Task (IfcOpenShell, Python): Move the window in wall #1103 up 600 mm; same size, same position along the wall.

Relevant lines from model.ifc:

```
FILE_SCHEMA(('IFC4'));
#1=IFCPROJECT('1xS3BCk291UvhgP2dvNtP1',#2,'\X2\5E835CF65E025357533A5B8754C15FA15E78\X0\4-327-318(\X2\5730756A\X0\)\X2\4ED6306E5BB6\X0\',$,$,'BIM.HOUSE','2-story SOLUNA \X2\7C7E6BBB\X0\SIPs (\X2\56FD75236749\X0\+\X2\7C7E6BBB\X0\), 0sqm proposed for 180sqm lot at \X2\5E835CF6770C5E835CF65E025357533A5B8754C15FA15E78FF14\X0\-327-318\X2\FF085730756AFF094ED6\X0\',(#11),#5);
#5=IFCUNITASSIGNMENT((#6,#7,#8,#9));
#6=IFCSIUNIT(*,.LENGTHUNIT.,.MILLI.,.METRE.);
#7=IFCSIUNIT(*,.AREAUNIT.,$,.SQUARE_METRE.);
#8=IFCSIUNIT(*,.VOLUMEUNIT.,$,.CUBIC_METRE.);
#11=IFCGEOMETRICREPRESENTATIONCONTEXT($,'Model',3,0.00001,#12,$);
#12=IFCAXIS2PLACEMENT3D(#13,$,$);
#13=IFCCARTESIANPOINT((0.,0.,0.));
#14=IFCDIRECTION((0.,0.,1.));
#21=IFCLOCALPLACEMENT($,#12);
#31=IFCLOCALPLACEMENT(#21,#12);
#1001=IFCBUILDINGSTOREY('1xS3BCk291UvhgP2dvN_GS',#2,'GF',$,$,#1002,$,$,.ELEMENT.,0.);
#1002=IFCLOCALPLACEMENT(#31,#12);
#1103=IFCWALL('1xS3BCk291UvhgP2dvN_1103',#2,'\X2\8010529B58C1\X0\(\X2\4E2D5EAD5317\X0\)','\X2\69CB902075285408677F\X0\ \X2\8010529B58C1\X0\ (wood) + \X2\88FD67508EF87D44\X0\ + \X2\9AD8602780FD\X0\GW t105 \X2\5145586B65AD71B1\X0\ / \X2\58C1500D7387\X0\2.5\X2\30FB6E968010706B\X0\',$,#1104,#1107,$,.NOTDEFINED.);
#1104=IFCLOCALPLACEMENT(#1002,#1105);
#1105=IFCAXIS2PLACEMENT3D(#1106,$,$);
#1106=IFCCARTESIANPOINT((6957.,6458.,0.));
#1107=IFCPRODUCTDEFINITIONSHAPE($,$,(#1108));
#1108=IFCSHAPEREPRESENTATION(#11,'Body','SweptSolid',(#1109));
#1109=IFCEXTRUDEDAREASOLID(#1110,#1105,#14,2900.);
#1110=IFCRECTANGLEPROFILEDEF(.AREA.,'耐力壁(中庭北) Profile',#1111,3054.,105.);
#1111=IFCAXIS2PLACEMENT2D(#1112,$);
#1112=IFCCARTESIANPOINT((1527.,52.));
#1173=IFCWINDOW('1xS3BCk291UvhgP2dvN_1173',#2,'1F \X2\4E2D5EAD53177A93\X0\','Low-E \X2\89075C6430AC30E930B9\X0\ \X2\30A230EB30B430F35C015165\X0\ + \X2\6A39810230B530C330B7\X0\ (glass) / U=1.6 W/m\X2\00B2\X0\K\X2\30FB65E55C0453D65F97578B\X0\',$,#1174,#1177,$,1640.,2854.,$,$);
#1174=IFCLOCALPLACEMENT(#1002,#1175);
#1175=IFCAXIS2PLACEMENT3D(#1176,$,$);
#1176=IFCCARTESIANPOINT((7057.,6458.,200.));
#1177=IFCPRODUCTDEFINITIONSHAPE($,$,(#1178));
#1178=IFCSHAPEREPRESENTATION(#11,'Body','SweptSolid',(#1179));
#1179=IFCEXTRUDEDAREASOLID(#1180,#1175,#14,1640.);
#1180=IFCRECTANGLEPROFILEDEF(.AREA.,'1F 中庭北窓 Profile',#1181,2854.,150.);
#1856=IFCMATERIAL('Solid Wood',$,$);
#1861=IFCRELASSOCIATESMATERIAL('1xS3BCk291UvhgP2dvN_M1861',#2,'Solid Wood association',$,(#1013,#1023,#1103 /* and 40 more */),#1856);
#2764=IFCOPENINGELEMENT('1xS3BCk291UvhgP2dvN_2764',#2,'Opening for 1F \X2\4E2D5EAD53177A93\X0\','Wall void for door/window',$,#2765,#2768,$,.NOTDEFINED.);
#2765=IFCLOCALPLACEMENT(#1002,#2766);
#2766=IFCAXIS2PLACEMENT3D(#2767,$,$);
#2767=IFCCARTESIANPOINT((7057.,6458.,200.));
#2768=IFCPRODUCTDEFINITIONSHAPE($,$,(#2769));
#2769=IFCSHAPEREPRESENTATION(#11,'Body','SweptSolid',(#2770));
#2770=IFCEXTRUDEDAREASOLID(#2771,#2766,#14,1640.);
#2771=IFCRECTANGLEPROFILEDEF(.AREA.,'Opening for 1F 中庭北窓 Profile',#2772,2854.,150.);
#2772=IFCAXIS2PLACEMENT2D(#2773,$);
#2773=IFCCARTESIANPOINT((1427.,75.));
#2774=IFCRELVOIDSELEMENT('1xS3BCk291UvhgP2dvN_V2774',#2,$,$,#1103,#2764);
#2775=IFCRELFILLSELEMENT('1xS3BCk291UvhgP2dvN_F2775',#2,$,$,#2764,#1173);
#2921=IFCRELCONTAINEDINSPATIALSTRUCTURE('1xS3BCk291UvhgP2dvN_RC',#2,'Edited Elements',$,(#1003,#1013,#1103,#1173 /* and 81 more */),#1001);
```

```python
import numpy as np
import ifcopenshell
import ifcopenshell.api.geometry
import ifcopenshell.util.placement
import ifcopenshell.util.unit

model = ifcopenshell.open("model.ifc")
unit_scale = ifcopenshell.util.unit.calculate_unit_scale(model)

window = model.by_id(1173)
opening = window.FillsVoids[0].RelatingOpeningElement
dz = 0.6 / unit_scale

shift = np.array([0.0, 0.0, dz])
# The window is not placed relative to its opening, so move both.
for product in (opening, window):
    matrix = ifcopenshell.util.placement.get_local_placement(product.ObjectPlacement)
    matrix[:3, 3] += shift
    ifcopenshell.api.geometry.edit_object_placement(model, product=product, matrix=matrix, is_si=False)

print(f"moved by {dz * unit_scale:+.3f} m")

model.write("model_rev.ifc")
```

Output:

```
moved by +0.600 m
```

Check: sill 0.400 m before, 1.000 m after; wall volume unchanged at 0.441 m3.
